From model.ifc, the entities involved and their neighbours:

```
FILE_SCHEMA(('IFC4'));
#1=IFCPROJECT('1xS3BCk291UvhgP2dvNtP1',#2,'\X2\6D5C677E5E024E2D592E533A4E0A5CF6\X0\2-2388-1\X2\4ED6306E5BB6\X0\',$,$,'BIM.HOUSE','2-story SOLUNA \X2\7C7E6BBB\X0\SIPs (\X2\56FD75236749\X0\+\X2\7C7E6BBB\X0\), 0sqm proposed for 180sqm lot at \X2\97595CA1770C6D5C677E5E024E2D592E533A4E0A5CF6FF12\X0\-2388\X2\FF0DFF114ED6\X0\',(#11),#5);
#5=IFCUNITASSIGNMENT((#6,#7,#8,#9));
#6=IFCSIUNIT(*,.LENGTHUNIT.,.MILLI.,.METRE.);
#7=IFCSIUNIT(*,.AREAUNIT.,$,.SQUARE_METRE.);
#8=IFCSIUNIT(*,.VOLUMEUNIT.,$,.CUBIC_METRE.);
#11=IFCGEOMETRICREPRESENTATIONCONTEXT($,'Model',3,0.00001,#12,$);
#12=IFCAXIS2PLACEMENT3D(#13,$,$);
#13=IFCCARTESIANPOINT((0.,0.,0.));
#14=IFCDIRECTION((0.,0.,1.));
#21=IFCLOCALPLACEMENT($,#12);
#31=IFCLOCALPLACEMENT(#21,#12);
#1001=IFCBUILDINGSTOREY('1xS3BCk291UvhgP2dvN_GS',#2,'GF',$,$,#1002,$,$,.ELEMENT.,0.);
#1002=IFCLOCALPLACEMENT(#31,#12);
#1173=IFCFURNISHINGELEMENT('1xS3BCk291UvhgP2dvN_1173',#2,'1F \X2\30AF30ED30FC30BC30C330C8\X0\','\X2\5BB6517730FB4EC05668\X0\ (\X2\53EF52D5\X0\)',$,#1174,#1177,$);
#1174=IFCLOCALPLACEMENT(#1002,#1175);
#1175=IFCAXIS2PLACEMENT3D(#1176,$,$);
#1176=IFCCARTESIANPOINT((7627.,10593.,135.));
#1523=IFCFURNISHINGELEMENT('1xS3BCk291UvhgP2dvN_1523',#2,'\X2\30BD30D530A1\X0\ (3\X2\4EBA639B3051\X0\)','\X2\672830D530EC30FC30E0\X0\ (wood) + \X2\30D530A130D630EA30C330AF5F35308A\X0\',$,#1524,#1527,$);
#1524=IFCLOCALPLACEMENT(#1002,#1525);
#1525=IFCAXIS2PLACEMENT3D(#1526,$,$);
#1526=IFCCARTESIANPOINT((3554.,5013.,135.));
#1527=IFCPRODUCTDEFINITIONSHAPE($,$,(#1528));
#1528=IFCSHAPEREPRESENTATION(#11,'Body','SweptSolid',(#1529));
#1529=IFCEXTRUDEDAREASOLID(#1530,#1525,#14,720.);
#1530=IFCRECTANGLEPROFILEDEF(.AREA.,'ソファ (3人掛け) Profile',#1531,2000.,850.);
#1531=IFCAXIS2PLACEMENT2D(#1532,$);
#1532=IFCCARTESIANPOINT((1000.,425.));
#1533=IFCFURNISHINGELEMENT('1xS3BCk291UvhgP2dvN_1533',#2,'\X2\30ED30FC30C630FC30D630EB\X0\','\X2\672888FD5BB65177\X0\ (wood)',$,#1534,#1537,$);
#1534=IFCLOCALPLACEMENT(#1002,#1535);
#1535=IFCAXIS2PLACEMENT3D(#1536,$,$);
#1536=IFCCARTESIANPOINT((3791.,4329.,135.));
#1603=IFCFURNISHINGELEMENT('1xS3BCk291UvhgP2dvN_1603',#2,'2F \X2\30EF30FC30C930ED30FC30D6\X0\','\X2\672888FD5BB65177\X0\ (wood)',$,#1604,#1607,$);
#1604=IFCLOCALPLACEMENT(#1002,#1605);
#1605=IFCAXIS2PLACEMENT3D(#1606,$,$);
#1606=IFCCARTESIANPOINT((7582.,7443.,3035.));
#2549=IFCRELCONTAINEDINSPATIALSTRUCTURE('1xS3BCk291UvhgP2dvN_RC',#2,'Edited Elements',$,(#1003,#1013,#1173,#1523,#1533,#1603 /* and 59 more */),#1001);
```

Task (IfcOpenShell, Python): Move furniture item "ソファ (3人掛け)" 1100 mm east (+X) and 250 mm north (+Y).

```python
import ifcopenshell
import ifcopenshell.api.geometry
import ifcopenshell.util.placement
import ifcopenshell.util.unit

model = ifcopenshell.open("model.ifc")
unit_scale = ifcopenshell.util.unit.calculate_unit_scale(model)

item = model.by_guid("1xS3BCk291UvhgP2dvN_1523")
matrix = ifcopenshell.util.placement.get_local_placement(item.ObjectPlacement)
matrix[0, 3] += 1.1 / unit_scale
matrix[1, 3] += 0.25 / unit_scale
ifcopenshell.api.geometry.edit_object_placement(model, product=item, matrix=matrix, is_si=False)

print(ifcopenshell.util.placement.get_local_placement(item.ObjectPlacement).round(3) + 0.0)

model.write("model-out.ifc")
```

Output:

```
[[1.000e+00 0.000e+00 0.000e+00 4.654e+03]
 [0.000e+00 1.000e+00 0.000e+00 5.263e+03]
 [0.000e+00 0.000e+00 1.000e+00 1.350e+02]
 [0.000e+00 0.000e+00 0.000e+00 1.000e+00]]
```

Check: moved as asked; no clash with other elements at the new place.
